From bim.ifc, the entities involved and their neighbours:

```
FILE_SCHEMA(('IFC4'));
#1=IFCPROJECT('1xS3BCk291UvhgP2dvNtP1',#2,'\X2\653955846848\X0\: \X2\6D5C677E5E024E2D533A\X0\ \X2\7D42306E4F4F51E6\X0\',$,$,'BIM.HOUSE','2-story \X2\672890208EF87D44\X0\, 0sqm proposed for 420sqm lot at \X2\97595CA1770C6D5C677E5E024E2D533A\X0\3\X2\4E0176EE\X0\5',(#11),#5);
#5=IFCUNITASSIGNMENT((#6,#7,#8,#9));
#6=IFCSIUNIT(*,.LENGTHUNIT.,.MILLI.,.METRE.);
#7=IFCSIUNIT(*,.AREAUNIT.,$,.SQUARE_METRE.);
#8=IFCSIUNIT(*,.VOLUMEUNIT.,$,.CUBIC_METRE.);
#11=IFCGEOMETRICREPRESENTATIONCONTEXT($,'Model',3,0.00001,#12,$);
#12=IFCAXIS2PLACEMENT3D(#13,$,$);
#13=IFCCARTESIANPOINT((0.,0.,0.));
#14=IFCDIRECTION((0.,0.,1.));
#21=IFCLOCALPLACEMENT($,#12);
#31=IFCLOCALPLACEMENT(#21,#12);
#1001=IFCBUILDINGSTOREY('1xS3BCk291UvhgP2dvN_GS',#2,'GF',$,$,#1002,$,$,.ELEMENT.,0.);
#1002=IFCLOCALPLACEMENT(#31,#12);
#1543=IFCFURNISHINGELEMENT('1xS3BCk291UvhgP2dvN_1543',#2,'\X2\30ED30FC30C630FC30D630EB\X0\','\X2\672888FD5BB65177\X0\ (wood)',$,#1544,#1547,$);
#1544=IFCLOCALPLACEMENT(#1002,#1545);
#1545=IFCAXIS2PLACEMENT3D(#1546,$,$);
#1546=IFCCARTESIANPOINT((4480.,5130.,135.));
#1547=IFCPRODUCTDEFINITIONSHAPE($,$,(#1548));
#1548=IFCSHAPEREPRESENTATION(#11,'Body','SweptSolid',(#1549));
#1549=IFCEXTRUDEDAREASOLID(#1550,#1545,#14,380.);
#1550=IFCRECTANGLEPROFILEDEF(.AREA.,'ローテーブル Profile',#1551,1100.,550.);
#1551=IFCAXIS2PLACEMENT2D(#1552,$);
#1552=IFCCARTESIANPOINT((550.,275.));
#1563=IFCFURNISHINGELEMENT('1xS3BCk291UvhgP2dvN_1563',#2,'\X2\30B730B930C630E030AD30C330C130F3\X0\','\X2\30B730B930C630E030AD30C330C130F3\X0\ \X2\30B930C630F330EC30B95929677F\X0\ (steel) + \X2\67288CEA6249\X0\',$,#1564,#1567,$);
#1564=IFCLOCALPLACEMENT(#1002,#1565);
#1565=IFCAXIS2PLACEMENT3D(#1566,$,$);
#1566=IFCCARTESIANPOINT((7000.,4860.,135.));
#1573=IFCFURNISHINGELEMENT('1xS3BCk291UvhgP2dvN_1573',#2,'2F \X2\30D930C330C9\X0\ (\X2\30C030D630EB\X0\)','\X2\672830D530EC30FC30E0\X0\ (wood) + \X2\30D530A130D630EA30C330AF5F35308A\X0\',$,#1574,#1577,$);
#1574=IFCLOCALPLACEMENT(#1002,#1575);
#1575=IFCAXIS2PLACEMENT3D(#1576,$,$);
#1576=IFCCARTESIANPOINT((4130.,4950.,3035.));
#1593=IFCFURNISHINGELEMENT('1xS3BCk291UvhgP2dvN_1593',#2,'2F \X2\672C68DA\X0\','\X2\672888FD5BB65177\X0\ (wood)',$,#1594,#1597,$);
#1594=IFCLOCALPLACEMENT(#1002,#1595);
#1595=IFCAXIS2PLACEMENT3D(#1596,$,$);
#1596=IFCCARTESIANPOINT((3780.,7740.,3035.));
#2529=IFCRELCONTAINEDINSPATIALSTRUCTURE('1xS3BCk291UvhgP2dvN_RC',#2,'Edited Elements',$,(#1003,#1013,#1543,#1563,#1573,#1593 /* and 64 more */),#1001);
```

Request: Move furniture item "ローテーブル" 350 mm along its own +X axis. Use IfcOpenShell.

```python
import ifcopenshell
import ifcopenshell.api.geometry
import ifcopenshell.util.placement
import ifcopenshell.util.unit

model = ifcopenshell.open("bim.ifc")
unit_scale = ifcopenshell.util.unit.calculate_unit_scale(model)

item = model.by_guid("1xS3BCk291UvhgP2dvN_1543")
matrix = ifcopenshell.util.placement.get_local_placement(item.ObjectPlacement)
matrix[:3, 3] += matrix[:3, 0] * 0.35 / unit_scale
ifcopenshell.api.geometry.edit_object_placement(model, product=item, matrix=matrix, is_si=False)

print(ifcopenshell.util.placement.get_local_placement(item.ObjectPlacement).round(3) + 0.0)

model.write("bim_v2.ifc")
```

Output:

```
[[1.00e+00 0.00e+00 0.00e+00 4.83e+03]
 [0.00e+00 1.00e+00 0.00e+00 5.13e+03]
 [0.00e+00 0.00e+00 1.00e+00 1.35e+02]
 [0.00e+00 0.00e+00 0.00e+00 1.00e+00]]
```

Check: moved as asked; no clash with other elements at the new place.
